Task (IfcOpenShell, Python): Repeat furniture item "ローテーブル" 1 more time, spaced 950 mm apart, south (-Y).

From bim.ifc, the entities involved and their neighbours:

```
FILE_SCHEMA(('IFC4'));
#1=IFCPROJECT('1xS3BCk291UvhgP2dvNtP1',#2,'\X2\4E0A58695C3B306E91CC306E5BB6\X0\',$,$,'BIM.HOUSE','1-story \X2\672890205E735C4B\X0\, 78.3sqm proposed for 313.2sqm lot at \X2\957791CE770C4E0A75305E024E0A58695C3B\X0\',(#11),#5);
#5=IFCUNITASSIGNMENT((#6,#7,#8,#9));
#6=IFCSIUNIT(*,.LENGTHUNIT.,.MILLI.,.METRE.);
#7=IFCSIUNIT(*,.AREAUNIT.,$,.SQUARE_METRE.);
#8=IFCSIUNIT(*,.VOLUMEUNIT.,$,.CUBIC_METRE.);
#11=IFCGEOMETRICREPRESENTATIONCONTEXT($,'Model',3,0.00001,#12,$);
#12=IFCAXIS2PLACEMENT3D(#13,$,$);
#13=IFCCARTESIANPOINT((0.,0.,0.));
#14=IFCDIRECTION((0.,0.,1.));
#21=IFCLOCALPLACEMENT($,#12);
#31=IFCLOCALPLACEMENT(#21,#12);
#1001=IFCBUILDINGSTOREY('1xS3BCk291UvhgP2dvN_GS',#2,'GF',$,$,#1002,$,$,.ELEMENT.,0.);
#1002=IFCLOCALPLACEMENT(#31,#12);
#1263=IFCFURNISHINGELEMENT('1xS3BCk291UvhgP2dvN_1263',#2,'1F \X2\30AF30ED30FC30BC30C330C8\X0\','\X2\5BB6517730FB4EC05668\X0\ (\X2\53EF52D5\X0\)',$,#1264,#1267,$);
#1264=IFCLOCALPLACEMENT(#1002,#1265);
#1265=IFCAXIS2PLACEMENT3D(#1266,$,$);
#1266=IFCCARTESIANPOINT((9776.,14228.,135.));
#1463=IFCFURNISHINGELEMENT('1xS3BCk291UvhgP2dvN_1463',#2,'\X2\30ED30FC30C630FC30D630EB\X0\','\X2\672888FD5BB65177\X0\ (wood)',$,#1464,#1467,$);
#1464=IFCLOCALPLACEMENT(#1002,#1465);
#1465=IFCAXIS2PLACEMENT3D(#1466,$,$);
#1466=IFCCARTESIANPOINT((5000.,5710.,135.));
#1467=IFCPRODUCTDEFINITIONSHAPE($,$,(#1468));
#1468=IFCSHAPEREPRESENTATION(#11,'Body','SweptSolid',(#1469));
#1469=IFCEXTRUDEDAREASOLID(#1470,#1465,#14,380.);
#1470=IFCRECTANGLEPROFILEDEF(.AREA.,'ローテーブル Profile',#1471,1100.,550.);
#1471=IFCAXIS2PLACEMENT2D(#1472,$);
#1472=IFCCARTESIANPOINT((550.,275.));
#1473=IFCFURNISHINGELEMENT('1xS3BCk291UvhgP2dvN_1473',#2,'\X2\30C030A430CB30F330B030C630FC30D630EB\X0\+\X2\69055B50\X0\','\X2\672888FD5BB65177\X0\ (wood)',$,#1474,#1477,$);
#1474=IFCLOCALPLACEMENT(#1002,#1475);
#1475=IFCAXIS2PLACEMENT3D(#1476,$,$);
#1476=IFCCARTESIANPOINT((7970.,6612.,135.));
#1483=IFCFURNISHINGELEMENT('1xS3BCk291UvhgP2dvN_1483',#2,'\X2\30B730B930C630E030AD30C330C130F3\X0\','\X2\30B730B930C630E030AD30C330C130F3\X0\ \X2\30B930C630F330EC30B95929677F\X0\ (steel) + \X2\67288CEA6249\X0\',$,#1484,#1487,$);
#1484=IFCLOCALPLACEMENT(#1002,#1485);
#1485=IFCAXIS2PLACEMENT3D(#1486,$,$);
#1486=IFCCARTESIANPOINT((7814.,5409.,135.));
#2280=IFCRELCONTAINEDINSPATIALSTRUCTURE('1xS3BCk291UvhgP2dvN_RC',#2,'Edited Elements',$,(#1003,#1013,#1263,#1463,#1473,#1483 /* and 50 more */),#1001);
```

```python
import numpy as np
import ifcopenshell
import ifcopenshell.api.geometry
import ifcopenshell.api.root
import ifcopenshell.util.element
import ifcopenshell.util.placement

model = ifcopenshell.open("bim.ifc")


def reuse_history(source, copy):
    """copy_class also copies each property set's owner history, people and application; keep the originals."""
    for rel in copy.IsDefinedBy:
        if rel.is_a("IfcRelDefinesByProperties") and (history := rel.RelatingPropertyDefinition.OwnerHistory):
            rel.RelatingPropertyDefinition.OwnerHistory = source.OwnerHistory
            ifcopenshell.util.element.remove_deep2(model, history)


source = model.by_id(1463)
base = ifcopenshell.util.placement.get_local_placement(source.ObjectPlacement)
step = np.array([0.0, -1.0, 0.0]) * 950.0

for i in range(1, 2):
    copy = ifcopenshell.api.root.copy_class(model, product=source)
    copy.Representation = ifcopenshell.util.element.copy_deep(
        model, source.Representation, exclude=["IfcGeometricRepresentationContext", "IfcRepresentationMap"]
    )
    reuse_history(source, copy)
    matrix = base.copy()
    matrix[:3, 3] += i * step
    print("added at", matrix[:3, 3].round(3) + 0.0)
    ifcopenshell.api.geometry.edit_object_placement(model, product=copy, matrix=matrix, is_si=False)

model.write("bim_rev.ifc")
```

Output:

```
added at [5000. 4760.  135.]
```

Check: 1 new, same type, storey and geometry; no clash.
